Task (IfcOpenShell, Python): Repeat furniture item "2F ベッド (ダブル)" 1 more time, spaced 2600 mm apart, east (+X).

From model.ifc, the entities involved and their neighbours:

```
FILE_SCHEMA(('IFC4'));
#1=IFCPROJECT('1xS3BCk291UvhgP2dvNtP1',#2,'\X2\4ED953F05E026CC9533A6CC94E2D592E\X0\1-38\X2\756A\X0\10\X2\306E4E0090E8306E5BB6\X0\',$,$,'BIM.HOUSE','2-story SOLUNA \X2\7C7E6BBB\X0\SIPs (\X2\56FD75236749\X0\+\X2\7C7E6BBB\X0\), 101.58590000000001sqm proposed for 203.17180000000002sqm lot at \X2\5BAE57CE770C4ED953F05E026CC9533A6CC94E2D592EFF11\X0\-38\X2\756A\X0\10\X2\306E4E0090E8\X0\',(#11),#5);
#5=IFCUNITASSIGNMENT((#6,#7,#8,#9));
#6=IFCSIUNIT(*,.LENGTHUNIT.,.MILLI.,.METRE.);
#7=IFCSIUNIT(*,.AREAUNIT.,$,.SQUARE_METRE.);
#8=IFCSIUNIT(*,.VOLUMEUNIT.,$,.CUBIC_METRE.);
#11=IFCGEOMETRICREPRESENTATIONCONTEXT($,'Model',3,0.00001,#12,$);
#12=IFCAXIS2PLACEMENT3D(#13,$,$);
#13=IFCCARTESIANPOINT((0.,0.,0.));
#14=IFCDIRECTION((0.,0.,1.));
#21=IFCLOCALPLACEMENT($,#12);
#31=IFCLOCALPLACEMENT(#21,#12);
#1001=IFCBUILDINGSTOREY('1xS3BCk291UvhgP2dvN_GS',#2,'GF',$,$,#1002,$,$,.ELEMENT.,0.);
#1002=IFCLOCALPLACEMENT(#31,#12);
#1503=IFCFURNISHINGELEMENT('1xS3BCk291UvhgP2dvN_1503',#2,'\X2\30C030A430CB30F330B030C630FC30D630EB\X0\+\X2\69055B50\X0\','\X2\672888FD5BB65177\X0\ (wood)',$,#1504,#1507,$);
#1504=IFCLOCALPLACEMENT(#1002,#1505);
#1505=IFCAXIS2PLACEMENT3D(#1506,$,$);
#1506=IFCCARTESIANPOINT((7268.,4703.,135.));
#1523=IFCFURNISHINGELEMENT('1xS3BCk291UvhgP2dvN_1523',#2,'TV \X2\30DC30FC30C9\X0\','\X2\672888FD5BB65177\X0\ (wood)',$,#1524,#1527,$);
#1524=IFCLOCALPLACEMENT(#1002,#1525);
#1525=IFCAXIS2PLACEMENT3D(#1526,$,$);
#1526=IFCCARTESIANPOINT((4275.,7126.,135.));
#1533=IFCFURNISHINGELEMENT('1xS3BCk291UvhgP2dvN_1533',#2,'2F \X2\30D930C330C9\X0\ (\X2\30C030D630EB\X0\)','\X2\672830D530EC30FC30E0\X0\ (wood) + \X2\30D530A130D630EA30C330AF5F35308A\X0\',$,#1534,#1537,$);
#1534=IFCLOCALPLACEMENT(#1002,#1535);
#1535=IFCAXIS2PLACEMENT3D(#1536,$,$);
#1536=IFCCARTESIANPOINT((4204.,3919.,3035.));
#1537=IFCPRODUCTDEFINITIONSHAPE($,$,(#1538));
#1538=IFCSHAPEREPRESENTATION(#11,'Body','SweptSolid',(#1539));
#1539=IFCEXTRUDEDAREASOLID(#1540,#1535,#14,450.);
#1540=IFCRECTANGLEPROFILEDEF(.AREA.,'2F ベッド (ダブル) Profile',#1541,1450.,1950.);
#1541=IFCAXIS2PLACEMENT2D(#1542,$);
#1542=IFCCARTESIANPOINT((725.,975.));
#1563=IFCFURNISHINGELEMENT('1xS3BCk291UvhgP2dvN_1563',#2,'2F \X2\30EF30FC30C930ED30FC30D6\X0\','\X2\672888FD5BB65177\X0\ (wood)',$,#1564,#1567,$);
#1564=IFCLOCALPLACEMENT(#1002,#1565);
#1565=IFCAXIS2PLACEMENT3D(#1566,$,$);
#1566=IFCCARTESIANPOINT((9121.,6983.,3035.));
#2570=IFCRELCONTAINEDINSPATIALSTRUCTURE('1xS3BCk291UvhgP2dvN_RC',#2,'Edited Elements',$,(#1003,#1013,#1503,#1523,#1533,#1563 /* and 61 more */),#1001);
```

```python
import numpy as np
import ifcopenshell
import ifcopenshell.api.geometry
import ifcopenshell.api.root
import ifcopenshell.util.element
import ifcopenshell.util.placement

model = ifcopenshell.open("model.ifc")


def reuse_history(source, copy):
    """copy_class also copies each property set's owner history, people and application; keep the originals."""
    for rel in copy.IsDefinedBy:
        if rel.is_a("IfcRelDefinesByProperties") and (history := rel.RelatingPropertyDefinition.OwnerHistory):
            rel.RelatingPropertyDefinition.OwnerHistory = source.OwnerHistory
            ifcopenshell.util.element.remove_deep2(model, history)


source = model.by_guid("1xS3BCk291UvhgP2dvN_1533")
base = ifcopenshell.util.placement.get_local_placement(source.ObjectPlacement)
step = np.array([1.0, 0.0, 0.0]) * 2600.0

for i in range(1, 2):
    copy = ifcopenshell.api.root.copy_class(model, product=source)
    copy.Representation = ifcopenshell.util.element.copy_deep(
        model, source.Representation, exclude=["IfcGeometricRepresentationContext", "IfcRepresentationMap"]
    )
    reuse_history(source, copy)
    matrix = base.copy()
    matrix[:3, 3] += i * step
    print("added at", matrix[:3, 3].round(3) + 0.0)
    ifcopenshell.api.geometry.edit_object_placement(model, product=copy, matrix=matrix, is_si=False)

model.write("model_rev.ifc")
```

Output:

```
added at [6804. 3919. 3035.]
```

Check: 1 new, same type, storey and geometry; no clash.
